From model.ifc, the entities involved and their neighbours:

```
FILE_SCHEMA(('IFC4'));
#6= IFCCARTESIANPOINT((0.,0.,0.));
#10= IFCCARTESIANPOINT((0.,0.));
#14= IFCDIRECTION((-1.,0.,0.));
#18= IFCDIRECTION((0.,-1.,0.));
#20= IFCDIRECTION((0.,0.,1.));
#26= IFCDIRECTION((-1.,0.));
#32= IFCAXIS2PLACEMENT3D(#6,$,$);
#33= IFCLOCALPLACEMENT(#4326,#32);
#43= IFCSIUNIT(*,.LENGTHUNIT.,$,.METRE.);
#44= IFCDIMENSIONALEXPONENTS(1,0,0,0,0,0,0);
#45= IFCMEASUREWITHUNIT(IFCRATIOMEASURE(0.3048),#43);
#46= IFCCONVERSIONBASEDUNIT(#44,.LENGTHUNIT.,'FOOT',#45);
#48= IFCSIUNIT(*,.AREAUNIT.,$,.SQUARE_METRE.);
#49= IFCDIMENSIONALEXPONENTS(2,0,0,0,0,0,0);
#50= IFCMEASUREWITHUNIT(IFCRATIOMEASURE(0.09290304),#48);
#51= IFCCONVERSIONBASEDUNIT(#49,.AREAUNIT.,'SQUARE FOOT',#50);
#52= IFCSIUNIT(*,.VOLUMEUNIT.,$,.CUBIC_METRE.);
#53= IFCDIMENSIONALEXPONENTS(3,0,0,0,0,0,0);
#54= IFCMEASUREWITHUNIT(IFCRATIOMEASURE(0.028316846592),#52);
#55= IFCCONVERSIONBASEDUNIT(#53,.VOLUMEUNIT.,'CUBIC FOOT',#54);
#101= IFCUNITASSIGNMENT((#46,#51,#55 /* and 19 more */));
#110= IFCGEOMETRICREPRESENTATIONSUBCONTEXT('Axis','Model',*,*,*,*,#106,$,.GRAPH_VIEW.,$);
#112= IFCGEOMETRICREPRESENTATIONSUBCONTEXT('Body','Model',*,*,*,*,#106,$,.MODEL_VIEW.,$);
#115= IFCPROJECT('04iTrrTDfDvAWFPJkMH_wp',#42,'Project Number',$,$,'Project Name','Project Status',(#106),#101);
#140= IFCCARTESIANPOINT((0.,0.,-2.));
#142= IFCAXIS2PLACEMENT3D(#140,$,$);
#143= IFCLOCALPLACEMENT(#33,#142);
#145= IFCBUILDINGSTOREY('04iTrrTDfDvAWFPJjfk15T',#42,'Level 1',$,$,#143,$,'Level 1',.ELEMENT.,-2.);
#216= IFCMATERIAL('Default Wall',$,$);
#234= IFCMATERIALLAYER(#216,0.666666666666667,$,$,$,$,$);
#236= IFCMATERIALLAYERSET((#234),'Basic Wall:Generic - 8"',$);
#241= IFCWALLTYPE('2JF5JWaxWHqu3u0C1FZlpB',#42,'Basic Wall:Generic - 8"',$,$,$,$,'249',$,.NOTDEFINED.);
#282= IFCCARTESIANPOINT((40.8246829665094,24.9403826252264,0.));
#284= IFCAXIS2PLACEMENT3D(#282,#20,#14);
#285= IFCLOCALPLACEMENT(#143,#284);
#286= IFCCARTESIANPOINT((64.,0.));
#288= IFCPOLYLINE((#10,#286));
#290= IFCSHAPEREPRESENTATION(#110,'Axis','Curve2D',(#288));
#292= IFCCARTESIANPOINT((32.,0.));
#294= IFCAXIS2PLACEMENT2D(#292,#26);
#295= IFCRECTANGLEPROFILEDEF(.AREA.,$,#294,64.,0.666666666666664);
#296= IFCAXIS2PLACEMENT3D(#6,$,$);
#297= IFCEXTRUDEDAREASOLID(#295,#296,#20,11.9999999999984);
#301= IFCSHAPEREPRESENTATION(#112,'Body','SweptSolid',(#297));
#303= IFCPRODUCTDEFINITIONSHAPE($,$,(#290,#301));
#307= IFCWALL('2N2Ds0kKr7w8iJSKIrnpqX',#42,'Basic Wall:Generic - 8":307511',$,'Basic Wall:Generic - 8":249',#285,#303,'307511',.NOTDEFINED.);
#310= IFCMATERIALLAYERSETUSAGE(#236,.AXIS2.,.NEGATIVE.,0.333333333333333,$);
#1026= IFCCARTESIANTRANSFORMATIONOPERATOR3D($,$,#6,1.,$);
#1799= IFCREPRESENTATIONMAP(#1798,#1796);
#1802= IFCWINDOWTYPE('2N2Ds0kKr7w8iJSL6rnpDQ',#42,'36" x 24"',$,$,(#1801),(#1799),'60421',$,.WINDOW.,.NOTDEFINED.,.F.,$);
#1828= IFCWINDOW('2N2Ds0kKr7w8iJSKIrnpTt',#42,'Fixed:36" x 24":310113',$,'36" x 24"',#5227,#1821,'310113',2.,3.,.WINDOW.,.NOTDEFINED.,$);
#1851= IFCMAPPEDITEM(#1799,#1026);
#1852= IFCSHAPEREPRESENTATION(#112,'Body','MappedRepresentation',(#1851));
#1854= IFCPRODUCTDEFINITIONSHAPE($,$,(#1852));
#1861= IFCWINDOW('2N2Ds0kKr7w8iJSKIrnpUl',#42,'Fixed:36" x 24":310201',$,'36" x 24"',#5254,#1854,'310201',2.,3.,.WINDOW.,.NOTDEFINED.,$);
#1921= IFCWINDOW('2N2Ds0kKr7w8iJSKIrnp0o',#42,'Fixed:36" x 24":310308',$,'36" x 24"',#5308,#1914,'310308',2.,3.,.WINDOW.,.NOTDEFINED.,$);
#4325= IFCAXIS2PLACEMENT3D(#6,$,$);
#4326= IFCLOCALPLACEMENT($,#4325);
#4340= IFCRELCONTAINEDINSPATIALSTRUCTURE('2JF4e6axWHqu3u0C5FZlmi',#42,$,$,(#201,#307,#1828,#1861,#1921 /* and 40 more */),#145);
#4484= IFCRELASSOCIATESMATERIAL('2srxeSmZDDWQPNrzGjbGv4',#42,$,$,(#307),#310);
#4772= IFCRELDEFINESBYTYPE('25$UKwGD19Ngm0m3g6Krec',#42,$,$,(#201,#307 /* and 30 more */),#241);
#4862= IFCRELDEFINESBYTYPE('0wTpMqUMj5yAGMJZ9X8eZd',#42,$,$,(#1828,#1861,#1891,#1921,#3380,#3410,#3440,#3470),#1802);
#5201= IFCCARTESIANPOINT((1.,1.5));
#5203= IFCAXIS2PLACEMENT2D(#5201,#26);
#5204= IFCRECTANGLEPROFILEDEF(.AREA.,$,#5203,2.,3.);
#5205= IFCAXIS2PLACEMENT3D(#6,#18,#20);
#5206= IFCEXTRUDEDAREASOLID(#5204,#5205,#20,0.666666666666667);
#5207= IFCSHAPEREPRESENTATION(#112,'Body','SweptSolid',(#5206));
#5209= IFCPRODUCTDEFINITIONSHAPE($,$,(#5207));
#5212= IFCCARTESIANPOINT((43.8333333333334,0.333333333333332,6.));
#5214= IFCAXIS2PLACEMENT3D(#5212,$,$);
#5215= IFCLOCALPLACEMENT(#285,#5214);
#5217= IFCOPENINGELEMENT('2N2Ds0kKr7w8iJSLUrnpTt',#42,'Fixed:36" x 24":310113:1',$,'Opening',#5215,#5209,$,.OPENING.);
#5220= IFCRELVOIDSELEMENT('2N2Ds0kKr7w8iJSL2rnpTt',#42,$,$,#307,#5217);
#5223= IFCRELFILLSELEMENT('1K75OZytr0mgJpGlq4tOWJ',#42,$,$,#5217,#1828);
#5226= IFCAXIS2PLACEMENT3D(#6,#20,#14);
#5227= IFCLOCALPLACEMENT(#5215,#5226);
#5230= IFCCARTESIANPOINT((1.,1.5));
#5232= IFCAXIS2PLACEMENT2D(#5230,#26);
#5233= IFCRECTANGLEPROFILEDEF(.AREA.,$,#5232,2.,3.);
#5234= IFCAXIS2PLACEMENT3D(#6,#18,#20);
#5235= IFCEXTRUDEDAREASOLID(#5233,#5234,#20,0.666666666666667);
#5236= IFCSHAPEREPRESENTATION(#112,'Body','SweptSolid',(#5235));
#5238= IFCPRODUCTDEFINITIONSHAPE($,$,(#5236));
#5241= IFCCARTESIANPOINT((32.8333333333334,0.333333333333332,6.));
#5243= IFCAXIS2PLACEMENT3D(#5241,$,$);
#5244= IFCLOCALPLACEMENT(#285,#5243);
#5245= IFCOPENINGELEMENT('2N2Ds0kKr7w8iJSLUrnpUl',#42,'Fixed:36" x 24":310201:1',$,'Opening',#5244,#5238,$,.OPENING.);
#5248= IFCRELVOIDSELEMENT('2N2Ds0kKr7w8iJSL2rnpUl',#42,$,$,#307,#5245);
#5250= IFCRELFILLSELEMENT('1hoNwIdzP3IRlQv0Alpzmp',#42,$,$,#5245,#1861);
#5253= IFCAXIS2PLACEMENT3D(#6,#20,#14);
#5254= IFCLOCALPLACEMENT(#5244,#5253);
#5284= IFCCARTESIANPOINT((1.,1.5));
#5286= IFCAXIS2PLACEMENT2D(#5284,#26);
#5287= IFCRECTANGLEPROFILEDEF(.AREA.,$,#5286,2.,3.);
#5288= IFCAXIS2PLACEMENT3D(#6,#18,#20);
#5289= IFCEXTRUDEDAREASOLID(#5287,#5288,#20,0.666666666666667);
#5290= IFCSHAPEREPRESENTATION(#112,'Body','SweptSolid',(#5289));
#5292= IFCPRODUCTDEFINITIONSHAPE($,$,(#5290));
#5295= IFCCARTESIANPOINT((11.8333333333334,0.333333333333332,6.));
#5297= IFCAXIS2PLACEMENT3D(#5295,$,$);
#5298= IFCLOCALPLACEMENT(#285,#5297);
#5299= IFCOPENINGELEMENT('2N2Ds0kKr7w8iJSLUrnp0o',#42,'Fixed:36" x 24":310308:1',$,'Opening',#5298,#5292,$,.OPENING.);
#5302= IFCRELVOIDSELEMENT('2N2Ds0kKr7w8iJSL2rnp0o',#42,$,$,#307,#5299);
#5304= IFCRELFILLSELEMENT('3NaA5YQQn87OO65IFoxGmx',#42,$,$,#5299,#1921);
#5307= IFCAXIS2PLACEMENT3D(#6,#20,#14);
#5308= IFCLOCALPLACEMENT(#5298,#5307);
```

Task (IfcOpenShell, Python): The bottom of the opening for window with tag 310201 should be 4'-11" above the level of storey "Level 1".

```python
import numpy as np
import ifcopenshell
import ifcopenshell.api.geometry
import ifcopenshell.geom
import ifcopenshell.util.element
import ifcopenshell.util.placement
import ifcopenshell.util.shape
import ifcopenshell.util.unit

model = ifcopenshell.open("model.ifc")
unit_scale = ifcopenshell.util.unit.calculate_unit_scale(model)

window = model.by_guid("2N2Ds0kKr7w8iJSKIrnpUl")
opening = window.FillsVoids[0].RelatingOpeningElement
storey = ifcopenshell.util.element.get_container(window, ifc_class="IfcBuildingStorey")
level = ifcopenshell.util.placement.get_local_placement(storey.ObjectPlacement)[2, 3]

# The opening's origin need not be at the sill, so measure its lowest point.
shape = ifcopenshell.geom.create_shape(ifcopenshell.geom.settings(), opening)
bottom = ifcopenshell.util.shape.get_shape_bottom_elevation(shape, shape.geometry) / unit_scale
dz = level + 59 * 0.0254 / unit_scale - bottom

shift = np.array([0.0, 0.0, dz])
# The window is placed relative to its opening, so it follows when the opening moves.
matrix = ifcopenshell.util.placement.get_local_placement(opening.ObjectPlacement)
matrix[:3, 3] += shift
ifcopenshell.api.geometry.edit_object_placement(
    model, product=opening, matrix=matrix, is_si=False, should_transform_children=True
)

print(f"moved by {dz * unit_scale:+.3f} m")

model.write("model_v2.ifc")
```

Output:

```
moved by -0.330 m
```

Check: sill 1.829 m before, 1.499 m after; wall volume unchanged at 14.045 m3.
